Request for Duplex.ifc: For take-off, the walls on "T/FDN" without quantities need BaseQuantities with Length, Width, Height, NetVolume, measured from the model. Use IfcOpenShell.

First a look at what the model holds.

```python
import ifcopenshell
import ifcopenshell.util.element
import ifcopenshell.util.unit

model = ifcopenshell.open("Duplex.ifc")
print(model.schema)
for unit_type in ("LENGTHUNIT", "AREAUNIT", "VOLUMEUNIT"):
    print(unit_type, ifcopenshell.util.unit.calculate_unit_scale(model, unit_type))
storey = next(s for s in model.by_type("IfcBuildingStorey") if s.Name == "T/FDN")
walls = [e for e in ifcopenshell.util.element.get_decomposition(storey) if e.is_a("IfcWall")]
for e in sorted(walls, key=lambda e: e.id()):
    print(e.id(), e.is_a(), e.Name, list(ifcopenshell.util.element.get_psets(e, qtos_only=True)), sep=" | ")
```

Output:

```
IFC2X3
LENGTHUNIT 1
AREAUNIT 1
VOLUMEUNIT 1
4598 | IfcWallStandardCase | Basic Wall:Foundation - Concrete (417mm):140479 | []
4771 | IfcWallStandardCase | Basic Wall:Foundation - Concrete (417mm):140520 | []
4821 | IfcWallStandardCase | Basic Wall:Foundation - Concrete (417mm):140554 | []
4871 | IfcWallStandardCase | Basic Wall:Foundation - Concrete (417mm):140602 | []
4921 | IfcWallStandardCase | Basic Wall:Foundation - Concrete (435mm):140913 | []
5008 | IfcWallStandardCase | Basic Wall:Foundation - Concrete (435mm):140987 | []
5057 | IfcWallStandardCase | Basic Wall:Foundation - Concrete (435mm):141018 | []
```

```python
import ifcopenshell
import ifcopenshell.api.pset
import ifcopenshell.geom
import ifcopenshell.util.element
import ifcopenshell.util.shape
import ifcopenshell.util.unit

model = ifcopenshell.open("Duplex.ifc")
unit_scale = ifcopenshell.util.unit.calculate_unit_scale(model)
volume_scale = ifcopenshell.util.unit.calculate_unit_scale(model, "VOLUMEUNIT")
settings = ifcopenshell.geom.settings()

storey = next(s for s in model.by_type("IfcBuildingStorey") if s.Name == "T/FDN")
walls = [e for e in ifcopenshell.util.element.get_decomposition(storey) if e.is_a("IfcWall")]

for e in sorted(walls, key=lambda e: e.id()):
    if ifcopenshell.util.element.get_psets(e, qtos_only=True, should_inherit=False):
        continue
    # Geometry comes back in metres, in the element's own axes.
    shape = ifcopenshell.geom.create_shape(settings, e)
    values = {
        "Length": ifcopenshell.util.shape.get_x(shape.geometry) / unit_scale,
        "Width": ifcopenshell.util.shape.get_y(shape.geometry) / unit_scale,
        "Height": ifcopenshell.util.shape.get_z(shape.geometry) / unit_scale,
        "NetVolume": ifcopenshell.util.shape.get_volume(shape.geometry) / volume_scale,
    }
    qto = ifcopenshell.api.pset.add_qto(model, product=e, name="BaseQuantities")
    ifcopenshell.api.pset.edit_qto(model, qto=qto, properties=values)
    print(e.id(), {k: round(v, 3) for k, v in values.items()})

model.write("Duplex_updated.ifc")
```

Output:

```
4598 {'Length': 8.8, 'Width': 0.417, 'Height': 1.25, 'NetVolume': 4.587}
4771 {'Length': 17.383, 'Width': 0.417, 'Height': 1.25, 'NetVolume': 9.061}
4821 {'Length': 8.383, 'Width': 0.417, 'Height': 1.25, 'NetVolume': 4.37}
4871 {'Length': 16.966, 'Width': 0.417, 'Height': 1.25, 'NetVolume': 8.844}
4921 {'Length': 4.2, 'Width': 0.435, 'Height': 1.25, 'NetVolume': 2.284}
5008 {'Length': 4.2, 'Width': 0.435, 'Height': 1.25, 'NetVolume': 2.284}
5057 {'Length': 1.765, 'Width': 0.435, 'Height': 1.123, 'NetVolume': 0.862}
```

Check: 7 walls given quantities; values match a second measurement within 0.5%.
